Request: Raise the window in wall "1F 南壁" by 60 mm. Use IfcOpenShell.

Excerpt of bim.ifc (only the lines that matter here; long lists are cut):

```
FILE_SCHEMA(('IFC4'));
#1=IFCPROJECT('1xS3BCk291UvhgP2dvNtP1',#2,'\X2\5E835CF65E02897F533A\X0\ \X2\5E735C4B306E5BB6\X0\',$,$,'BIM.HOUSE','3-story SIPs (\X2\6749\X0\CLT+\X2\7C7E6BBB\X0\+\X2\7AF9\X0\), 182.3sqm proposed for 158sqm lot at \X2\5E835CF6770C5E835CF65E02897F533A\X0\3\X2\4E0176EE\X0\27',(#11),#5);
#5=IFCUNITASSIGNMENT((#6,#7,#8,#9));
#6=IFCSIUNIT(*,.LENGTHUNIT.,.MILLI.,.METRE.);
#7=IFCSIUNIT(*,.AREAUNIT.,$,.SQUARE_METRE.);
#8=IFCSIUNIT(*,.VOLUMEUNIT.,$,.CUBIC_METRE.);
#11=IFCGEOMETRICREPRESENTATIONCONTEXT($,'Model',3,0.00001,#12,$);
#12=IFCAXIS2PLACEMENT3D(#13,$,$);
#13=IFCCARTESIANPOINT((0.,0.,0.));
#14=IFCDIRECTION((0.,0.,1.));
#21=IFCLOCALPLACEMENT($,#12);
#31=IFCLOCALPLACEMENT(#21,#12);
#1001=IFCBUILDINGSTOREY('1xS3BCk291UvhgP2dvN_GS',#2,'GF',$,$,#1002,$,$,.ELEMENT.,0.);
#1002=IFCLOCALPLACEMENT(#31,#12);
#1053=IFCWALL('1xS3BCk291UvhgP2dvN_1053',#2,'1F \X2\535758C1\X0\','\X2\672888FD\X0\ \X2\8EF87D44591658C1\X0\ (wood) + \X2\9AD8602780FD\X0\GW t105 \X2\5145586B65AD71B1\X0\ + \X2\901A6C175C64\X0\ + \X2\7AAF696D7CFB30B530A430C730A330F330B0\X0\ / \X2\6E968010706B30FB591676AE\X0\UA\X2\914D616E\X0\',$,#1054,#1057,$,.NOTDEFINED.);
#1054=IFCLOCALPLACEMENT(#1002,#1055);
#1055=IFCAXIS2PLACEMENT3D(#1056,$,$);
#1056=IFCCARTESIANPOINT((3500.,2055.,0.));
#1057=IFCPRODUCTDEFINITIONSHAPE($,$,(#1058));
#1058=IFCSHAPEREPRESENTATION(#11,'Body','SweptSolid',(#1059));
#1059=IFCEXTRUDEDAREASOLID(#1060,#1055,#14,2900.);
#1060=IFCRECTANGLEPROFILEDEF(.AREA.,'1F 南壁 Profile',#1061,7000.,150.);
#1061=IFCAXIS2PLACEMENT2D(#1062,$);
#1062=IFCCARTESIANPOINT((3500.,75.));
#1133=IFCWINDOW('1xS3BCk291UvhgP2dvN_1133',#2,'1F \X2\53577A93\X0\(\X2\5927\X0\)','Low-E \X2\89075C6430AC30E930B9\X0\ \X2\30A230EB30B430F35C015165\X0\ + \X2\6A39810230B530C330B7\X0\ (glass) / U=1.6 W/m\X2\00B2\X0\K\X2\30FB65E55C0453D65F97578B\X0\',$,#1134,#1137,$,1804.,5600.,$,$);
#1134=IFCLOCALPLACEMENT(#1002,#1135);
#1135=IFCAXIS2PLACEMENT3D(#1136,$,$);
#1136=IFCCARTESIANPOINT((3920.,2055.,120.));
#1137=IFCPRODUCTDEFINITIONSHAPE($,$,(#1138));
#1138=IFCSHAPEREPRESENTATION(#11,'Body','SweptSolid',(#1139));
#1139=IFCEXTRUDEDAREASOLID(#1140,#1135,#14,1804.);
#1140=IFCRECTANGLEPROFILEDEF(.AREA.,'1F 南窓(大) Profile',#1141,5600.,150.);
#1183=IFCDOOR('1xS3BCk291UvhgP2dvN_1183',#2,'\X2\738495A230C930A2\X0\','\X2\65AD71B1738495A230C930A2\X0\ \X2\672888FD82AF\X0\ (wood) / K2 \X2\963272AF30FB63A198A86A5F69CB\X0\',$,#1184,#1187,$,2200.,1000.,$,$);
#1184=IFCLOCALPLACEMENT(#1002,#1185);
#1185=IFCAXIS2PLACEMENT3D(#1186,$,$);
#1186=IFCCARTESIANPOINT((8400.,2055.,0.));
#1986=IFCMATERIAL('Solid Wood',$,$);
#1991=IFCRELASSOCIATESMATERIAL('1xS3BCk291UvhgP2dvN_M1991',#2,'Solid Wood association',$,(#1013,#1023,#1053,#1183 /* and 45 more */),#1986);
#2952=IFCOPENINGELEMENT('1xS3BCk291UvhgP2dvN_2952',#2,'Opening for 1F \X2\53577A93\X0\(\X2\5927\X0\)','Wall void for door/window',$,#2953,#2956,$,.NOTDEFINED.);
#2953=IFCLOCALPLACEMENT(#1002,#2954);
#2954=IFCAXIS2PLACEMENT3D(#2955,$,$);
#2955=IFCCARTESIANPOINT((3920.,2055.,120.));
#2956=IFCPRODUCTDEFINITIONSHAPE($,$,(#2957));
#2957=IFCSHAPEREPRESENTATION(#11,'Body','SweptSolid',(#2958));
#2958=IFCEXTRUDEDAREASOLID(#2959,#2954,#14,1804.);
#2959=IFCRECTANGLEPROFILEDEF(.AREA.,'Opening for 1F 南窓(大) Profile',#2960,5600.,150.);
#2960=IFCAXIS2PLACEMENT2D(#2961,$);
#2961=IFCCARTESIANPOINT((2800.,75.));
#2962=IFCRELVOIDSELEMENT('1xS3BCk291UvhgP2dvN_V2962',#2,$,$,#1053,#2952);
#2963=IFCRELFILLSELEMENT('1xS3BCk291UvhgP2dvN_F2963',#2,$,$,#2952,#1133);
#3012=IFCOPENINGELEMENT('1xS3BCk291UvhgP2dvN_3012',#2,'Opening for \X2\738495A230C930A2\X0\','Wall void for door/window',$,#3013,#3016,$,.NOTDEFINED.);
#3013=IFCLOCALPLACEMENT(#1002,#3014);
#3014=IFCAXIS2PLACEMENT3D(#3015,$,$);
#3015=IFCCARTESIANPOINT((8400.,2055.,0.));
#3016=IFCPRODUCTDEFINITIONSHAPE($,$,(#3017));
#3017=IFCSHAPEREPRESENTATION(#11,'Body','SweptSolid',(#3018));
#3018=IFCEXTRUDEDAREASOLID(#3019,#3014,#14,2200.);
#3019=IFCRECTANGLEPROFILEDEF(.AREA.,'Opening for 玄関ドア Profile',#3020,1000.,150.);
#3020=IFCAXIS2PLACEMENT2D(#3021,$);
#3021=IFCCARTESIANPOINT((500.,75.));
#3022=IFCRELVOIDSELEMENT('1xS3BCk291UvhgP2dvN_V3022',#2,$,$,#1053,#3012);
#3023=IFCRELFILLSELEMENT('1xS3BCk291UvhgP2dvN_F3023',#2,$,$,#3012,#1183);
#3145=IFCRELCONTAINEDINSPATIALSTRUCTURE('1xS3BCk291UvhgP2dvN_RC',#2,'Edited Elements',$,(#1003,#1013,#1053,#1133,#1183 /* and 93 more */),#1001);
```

```python
import numpy as np
import ifcopenshell
import ifcopenshell.api.geometry
import ifcopenshell.util.placement
import ifcopenshell.util.unit

model = ifcopenshell.open("bim.ifc")
unit_scale = ifcopenshell.util.unit.calculate_unit_scale(model)

window = model.by_guid("1xS3BCk291UvhgP2dvN_1133")
opening = window.FillsVoids[0].RelatingOpeningElement
dz = 60.0

shift = np.array([0.0, 0.0, dz])
# The window is not placed relative to its opening, so move both.
for product in (opening, window):
    matrix = ifcopenshell.util.placement.get_local_placement(product.ObjectPlacement)
    matrix[:3, 3] += shift
    ifcopenshell.api.geometry.edit_object_placement(model, product=product, matrix=matrix, is_si=False)

print(f"moved by {dz * unit_scale:+.3f} m")

model.write("bim_rev.ifc")
```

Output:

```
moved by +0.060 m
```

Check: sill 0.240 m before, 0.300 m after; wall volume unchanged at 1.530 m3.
